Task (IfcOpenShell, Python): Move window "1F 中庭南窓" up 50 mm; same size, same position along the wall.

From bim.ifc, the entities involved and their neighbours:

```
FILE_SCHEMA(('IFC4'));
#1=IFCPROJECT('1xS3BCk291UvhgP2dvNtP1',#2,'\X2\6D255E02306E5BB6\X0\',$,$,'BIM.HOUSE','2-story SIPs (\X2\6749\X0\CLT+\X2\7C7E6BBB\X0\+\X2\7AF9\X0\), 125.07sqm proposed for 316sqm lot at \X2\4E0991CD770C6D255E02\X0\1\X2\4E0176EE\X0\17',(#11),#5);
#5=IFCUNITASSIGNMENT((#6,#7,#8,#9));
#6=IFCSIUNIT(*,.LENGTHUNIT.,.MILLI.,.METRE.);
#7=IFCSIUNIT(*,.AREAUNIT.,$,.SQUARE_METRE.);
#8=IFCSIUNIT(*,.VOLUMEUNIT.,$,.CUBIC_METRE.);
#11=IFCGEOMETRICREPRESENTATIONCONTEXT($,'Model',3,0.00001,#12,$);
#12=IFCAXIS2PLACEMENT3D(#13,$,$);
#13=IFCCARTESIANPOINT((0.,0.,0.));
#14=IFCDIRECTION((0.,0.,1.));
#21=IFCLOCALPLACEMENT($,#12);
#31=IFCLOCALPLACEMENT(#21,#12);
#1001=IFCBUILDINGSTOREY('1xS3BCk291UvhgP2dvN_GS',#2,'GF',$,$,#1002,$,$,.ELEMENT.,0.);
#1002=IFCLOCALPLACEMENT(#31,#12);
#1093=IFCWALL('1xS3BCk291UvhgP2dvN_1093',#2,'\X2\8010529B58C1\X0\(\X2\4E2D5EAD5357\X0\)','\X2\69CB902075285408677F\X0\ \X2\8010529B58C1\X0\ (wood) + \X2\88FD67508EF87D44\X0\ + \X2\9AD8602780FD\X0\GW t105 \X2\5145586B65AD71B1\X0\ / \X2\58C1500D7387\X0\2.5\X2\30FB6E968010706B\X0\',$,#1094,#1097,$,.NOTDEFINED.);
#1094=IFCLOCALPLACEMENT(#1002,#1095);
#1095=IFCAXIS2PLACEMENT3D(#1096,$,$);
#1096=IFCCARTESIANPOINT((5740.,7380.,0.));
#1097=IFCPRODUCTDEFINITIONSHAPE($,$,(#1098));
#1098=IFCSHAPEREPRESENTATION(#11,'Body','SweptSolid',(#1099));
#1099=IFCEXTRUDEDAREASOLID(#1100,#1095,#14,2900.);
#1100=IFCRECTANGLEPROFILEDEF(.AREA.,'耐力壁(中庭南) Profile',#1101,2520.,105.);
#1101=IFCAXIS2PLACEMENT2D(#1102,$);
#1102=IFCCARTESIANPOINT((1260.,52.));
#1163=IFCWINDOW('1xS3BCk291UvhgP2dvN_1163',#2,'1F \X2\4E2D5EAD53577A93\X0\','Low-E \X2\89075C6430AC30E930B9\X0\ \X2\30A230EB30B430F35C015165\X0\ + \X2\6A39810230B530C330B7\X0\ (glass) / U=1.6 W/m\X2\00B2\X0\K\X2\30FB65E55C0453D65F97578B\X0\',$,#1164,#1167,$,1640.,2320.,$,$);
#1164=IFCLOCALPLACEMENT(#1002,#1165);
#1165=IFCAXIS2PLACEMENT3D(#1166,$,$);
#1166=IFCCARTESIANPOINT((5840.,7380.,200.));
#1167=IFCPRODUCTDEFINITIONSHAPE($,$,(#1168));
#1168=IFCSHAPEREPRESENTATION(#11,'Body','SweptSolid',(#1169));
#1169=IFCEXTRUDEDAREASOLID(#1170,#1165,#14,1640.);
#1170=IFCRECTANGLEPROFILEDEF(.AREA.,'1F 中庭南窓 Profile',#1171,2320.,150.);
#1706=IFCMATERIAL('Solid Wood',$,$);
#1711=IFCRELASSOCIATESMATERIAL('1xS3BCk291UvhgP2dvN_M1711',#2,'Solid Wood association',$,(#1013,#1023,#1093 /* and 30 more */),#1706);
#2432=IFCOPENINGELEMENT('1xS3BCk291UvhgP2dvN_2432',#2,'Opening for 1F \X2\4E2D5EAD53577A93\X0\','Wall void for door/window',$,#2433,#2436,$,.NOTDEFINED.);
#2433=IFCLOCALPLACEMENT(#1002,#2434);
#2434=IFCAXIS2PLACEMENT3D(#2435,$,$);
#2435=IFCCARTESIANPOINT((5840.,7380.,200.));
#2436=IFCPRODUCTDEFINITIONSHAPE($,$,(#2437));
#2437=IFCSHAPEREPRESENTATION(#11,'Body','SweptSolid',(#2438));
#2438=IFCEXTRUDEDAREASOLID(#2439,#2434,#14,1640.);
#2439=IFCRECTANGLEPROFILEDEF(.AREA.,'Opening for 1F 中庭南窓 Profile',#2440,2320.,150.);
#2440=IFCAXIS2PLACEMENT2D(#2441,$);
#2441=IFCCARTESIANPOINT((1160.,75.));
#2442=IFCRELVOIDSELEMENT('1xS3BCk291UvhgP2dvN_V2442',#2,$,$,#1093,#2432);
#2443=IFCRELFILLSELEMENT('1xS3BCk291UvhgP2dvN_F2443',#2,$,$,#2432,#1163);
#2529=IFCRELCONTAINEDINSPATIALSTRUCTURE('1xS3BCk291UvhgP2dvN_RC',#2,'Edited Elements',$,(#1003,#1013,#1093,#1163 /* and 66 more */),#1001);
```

```python
import numpy as np
import ifcopenshell
import ifcopenshell.api.geometry
import ifcopenshell.util.placement
import ifcopenshell.util.unit

model = ifcopenshell.open("bim.ifc")
unit_scale = ifcopenshell.util.unit.calculate_unit_scale(model)

window = model.by_guid("1xS3BCk291UvhgP2dvN_1163")
opening = window.FillsVoids[0].RelatingOpeningElement
dz = 0.05 / unit_scale

shift = np.array([0.0, 0.0, dz])
# The window is not placed relative to its opening, so move both.
for product in (opening, window):
    matrix = ifcopenshell.util.placement.get_local_placement(product.ObjectPlacement)
    matrix[:3, 3] += shift
    ifcopenshell.api.geometry.edit_object_placement(model, product=product, matrix=matrix, is_si=False)

print(f"moved by {dz * unit_scale:+.3f} m")

model.write("bim_edited.ifc")
```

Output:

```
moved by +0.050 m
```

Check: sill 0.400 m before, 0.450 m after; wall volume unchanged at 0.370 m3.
